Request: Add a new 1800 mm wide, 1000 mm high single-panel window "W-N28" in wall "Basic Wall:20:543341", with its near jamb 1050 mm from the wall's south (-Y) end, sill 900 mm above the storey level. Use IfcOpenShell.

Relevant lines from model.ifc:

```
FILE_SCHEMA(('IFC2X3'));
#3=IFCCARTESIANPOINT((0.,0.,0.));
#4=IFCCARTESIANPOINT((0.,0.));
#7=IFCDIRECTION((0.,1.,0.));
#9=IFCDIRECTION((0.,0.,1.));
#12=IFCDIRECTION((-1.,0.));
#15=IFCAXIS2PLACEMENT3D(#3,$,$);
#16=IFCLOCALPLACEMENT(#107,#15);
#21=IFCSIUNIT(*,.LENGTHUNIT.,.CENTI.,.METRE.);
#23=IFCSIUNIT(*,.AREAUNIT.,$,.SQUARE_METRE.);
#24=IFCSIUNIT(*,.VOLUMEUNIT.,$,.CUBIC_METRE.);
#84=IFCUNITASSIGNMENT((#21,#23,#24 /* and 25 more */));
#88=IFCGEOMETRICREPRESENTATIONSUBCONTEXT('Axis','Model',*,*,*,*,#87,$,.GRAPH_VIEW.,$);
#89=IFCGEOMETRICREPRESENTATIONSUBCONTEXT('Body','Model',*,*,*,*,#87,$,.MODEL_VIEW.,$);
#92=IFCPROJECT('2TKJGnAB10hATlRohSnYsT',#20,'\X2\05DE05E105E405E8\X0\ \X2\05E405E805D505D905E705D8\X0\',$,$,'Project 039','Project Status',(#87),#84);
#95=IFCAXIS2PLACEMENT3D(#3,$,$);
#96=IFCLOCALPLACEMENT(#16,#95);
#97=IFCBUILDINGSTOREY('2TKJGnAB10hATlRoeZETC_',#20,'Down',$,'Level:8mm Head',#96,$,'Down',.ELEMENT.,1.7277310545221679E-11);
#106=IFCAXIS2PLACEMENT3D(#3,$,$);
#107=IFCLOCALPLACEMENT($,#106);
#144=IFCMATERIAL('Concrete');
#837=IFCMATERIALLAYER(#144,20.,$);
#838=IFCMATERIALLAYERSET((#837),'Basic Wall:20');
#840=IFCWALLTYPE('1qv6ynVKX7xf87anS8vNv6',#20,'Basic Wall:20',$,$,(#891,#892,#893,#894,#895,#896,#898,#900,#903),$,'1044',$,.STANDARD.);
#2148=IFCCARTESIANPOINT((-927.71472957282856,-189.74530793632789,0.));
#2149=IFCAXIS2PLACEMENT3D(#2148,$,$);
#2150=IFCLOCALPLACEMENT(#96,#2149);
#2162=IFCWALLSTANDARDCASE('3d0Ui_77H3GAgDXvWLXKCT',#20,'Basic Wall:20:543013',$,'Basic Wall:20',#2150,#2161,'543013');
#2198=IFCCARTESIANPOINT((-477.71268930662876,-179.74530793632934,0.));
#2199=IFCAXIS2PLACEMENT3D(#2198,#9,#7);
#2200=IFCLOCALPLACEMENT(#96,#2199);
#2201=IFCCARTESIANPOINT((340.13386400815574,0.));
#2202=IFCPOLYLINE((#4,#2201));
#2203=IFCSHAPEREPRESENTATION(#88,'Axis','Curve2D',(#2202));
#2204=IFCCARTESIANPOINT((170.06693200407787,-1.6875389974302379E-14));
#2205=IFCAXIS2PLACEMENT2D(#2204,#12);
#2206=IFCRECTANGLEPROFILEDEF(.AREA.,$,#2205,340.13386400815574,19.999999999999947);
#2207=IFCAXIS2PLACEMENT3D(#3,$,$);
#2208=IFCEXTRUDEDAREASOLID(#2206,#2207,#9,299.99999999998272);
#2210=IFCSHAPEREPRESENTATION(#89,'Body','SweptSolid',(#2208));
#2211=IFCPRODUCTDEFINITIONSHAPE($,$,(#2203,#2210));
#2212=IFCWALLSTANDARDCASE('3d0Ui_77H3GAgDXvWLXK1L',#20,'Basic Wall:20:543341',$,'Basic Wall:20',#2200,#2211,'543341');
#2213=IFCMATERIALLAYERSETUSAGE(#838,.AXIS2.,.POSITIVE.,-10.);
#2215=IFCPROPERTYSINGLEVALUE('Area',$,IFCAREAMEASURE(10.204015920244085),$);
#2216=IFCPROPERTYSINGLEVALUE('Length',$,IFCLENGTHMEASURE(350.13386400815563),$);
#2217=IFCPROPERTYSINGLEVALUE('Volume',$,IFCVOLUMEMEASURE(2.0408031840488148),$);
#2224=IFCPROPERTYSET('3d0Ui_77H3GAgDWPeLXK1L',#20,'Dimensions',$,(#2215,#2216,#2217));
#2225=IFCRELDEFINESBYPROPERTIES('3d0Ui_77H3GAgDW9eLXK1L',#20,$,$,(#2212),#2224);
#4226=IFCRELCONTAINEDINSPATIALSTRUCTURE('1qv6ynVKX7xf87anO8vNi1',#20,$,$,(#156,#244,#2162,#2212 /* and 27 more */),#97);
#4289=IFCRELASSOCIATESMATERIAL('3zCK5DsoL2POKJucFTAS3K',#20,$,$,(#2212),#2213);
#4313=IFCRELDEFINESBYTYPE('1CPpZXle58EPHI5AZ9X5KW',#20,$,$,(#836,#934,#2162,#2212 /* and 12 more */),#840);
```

```python
import numpy as np
import ifcopenshell
import ifcopenshell.api.feature
import ifcopenshell.api.geometry
import ifcopenshell.api.pset
import ifcopenshell.api.root
import ifcopenshell.api.spatial
import ifcopenshell.api.type
import ifcopenshell.geom
import ifcopenshell.util.element
import ifcopenshell.util.placement
import ifcopenshell.util.representation
import ifcopenshell.util.shape
import ifcopenshell.util.unit

model = ifcopenshell.open("model.ifc")
unit_scale = ifcopenshell.util.unit.calculate_unit_scale(model)
area_scale = ifcopenshell.util.unit.calculate_unit_scale(model, "AREAUNIT")
volume_scale = ifcopenshell.util.unit.calculate_unit_scale(model, "VOLUMEUNIT")
settings = ifcopenshell.geom.settings()


def volume(element):
    """Net volume in cubic metres, openings subtracted."""
    shape = ifcopenshell.geom.create_shape(settings, element)
    return ifcopenshell.util.shape.get_volume(shape.geometry)


wall = model.by_guid("3d0Ui_77H3GAgDXvWLXK1L")
storey = ifcopenshell.util.element.get_container(wall, ifc_class="IfcBuildingStorey")
context = ifcopenshell.util.representation.get_context(model, "Model", "Body", "MODEL_VIEW")
before = volume(wall)

width, height, from_end, sill = 1.8, 1, 1.05, 0.9  # metres

# The wall runs along its own X axis, and the end named is its -X end.
wall_shape = ifcopenshell.geom.create_shape(settings, wall)
x, y, z = ifcopenshell.util.shape.get_vertices(wall_shape.geometry).T
start = x.min() + from_end
face, thickness = float(y.min()), float(y.max() - y.min())
wall_matrix = ifcopenshell.util.placement.get_local_placement(wall.ObjectPlacement)
level = ifcopenshell.util.placement.get_local_placement(storey.ObjectPlacement)[2, 3]


def in_wall(x, y):
    """Placement at x, y metres in the wall's axes, at sill height."""
    matrix = wall_matrix.copy()
    matrix[:, 3] = wall_matrix @ np.array([x / unit_scale, y / unit_scale, 0.0, 1.0])
    matrix[2, 3] = level + sill / unit_scale
    return matrix


# Opening: a box that overshoots both wall faces by 50 mm.
opening = ifcopenshell.api.root.create_entity(model, ifc_class="IfcOpeningElement")
box = ifcopenshell.api.geometry.add_wall_representation(
    model, context=context, length=width, height=height, thickness=thickness + 0.1
)
ifcopenshell.api.geometry.assign_representation(model, product=opening, representation=box)
ifcopenshell.api.geometry.edit_object_placement(model, product=opening, matrix=in_wall(start, face - 0.05), is_si=False)
ifcopenshell.api.feature.add_feature(model, feature=opening, element=wall)

window = ifcopenshell.api.root.create_entity(model, ifc_class="IfcWindow", name="W-N28")
window.OverallWidth, window.OverallHeight = width / unit_scale, height / unit_scale
body = ifcopenshell.api.geometry.add_window_representation(
    model,
    context=context,
    overall_width=window.OverallWidth,
    overall_height=window.OverallHeight,
    partition_type="SINGLE_PANEL",
)
ifcopenshell.api.geometry.assign_representation(model, product=window, representation=body)
ifcopenshell.api.spatial.assign_container(model, products=[window], relating_structure=storey)
fills = ifcopenshell.api.feature.add_filling(model, opening=opening, element=window)
fills.OwnerHistory = window.OwnerHistory  # required in IFC2X3

# IFC2X3 keeps the operation on the window style.
style = ifcopenshell.api.root.create_entity(model, ifc_class="IfcWindowStyle", name="W-N28")
style.OperationType, style.ConstructionType = "SINGLE_PANEL", "NOTDEFINED"
style.ParameterTakesPrecedence = style.Sizeable = False
ifcopenshell.api.type.assign_type(model, related_objects=[window], relating_type=style)

# Centre the window in the wall's thickness.
ifcopenshell.api.geometry.edit_object_placement(model, product=window, matrix=in_wall(start, face), is_si=False)
window_shape = ifcopenshell.geom.create_shape(settings, window)
depth = ifcopenshell.util.shape.get_vertices(window_shape.geometry)[:, 1]
offset = face + thickness / 2 - (depth.min() + depth.max()) / 2
ifcopenshell.api.geometry.edit_object_placement(model, product=window, matrix=in_wall(start, offset), is_si=False)

after = volume(wall)

# Update the wall's stored quantities.
pset = model.by_id(ifcopenshell.util.element.get_pset(wall, "Dimensions", should_inherit=False)["id"])
ifcopenshell.api.pset.edit_pset(model, pset=pset, properties={
    "Area": model.create_entity("IfcAreaMeasure", after / thickness / area_scale),
    "Volume": model.create_entity("IfcVolumeMeasure", after / volume_scale),
})

print(f"wall volume {before:.3f} -> {after:.3f} m3")

model.write("model_v2.ifc")
```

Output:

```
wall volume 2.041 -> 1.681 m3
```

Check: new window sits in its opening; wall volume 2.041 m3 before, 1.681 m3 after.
